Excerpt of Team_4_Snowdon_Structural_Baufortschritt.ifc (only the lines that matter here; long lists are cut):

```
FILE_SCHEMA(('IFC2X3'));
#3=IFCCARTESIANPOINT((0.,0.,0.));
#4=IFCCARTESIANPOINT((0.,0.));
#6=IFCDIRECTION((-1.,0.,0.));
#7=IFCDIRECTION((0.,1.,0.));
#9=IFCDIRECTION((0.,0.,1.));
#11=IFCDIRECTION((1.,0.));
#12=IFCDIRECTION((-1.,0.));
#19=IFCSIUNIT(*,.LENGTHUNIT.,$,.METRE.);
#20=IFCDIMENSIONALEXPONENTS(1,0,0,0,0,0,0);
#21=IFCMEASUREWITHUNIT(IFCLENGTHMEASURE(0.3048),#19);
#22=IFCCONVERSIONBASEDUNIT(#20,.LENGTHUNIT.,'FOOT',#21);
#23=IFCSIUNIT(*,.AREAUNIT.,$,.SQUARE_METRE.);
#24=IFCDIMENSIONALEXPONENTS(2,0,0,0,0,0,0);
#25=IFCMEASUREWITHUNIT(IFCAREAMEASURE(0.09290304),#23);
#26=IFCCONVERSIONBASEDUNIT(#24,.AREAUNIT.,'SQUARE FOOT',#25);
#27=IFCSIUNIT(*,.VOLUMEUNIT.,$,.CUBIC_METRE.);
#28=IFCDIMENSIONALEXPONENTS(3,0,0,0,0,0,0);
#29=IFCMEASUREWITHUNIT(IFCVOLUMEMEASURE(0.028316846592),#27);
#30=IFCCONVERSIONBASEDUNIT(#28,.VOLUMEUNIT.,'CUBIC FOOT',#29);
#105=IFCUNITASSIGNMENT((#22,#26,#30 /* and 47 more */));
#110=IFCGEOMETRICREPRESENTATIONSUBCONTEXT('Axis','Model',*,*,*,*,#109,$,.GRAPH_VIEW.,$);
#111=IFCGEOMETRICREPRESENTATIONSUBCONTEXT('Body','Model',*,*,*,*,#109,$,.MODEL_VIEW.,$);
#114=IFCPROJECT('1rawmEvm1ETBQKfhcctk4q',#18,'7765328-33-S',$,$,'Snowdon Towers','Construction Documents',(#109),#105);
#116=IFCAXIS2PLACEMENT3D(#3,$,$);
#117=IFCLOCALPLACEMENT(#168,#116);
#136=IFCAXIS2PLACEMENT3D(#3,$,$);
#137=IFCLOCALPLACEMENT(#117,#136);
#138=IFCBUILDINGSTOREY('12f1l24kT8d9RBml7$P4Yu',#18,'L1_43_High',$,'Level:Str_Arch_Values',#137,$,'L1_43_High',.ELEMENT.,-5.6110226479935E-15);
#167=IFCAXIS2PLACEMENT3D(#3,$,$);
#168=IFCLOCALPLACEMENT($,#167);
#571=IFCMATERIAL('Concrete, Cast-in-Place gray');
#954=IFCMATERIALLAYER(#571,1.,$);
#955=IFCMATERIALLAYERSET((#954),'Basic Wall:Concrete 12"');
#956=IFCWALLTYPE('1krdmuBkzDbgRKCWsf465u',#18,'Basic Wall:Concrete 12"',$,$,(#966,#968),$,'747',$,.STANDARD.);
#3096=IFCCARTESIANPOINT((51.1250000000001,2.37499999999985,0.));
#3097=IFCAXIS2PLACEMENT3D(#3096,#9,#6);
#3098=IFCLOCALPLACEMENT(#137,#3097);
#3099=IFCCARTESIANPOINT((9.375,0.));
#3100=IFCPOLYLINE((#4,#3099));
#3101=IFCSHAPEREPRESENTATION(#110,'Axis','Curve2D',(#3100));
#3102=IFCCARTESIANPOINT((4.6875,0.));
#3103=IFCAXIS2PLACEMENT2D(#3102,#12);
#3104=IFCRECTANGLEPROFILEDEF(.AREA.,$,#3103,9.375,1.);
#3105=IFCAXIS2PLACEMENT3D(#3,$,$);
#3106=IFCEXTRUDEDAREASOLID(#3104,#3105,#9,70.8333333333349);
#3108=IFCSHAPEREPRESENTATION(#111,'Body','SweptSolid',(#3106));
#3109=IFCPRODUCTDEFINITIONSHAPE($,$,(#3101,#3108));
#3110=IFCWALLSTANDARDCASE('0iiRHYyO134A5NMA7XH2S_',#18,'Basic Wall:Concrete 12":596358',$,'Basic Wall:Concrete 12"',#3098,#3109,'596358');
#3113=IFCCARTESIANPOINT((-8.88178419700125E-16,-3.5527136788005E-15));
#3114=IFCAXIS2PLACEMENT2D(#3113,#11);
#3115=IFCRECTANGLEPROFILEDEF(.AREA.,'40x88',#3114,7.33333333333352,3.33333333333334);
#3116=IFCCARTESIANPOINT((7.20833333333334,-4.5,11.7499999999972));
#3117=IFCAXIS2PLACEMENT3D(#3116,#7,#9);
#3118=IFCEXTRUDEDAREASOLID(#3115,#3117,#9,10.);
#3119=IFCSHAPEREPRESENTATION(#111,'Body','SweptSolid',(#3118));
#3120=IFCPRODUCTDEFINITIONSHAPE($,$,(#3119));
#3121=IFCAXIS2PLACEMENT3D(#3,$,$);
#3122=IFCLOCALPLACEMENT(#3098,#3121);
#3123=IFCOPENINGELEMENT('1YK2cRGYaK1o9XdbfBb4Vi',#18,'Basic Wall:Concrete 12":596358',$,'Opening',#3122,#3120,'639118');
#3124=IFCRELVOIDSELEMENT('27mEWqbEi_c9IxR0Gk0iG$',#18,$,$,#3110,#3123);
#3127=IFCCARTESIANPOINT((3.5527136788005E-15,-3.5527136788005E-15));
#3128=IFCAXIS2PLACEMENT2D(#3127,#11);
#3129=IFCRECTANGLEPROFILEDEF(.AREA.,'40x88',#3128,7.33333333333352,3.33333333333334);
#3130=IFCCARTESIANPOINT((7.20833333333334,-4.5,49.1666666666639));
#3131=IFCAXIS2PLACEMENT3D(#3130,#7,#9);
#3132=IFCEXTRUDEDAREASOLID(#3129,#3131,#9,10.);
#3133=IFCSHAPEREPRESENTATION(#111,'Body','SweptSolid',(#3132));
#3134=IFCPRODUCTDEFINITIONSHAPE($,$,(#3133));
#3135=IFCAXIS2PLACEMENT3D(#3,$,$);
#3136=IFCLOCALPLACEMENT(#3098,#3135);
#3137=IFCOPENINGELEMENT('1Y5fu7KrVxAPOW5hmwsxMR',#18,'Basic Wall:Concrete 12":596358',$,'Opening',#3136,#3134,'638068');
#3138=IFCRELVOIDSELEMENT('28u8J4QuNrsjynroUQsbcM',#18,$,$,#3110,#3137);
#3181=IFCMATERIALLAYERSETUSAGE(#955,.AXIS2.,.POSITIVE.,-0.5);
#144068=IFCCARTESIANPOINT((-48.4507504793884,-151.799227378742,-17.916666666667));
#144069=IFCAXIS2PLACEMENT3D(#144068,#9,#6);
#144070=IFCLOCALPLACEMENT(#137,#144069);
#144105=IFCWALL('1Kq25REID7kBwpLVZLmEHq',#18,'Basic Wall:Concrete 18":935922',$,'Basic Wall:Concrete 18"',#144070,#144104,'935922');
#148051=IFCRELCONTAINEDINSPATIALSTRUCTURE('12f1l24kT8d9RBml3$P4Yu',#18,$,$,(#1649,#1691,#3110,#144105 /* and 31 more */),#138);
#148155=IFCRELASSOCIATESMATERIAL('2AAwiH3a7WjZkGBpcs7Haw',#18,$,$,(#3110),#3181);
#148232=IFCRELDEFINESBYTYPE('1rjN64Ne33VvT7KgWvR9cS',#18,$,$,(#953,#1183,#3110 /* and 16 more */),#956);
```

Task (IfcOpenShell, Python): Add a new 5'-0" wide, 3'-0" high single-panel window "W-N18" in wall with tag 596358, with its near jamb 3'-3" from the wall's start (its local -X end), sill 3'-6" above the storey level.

```python
import numpy as np
import ifcopenshell
import ifcopenshell.api.feature
import ifcopenshell.api.geometry
import ifcopenshell.api.root
import ifcopenshell.api.spatial
import ifcopenshell.api.type
import ifcopenshell.geom
import ifcopenshell.util.element
import ifcopenshell.util.placement
import ifcopenshell.util.representation
import ifcopenshell.util.shape
import ifcopenshell.util.unit

model = ifcopenshell.open("Team_4_Snowdon_Structural_Baufortschritt.ifc")
unit_scale = ifcopenshell.util.unit.calculate_unit_scale(model)
settings = ifcopenshell.geom.settings()


def volume(element):
    """Net volume in cubic metres, openings subtracted."""
    shape = ifcopenshell.geom.create_shape(settings, element)
    return ifcopenshell.util.shape.get_volume(shape.geometry)


wall = model.by_guid("0iiRHYyO134A5NMA7XH2S_")
storey = ifcopenshell.util.element.get_container(wall, ifc_class="IfcBuildingStorey")
context = ifcopenshell.util.representation.get_context(model, "Model", "Body", "MODEL_VIEW")
before = volume(wall)

width, height, from_end, sill = 1.524, 0.9144, 0.9906, 1.0668  # metres

# The wall runs along its own X axis, and the end named is its -X end.
wall_shape = ifcopenshell.geom.create_shape(settings, wall)
x, y, z = ifcopenshell.util.shape.get_vertices(wall_shape.geometry).T
start = x.min() + from_end
face, thickness = float(y.min()), float(y.max() - y.min())
wall_matrix = ifcopenshell.util.placement.get_local_placement(wall.ObjectPlacement)
level = ifcopenshell.util.placement.get_local_placement(storey.ObjectPlacement)[2, 3]


def in_wall(x, y):
    """Placement at x, y metres in the wall's axes, at sill height."""
    matrix = wall_matrix.copy()
    matrix[:, 3] = wall_matrix @ np.array([x / unit_scale, y / unit_scale, 0.0, 1.0])
    matrix[2, 3] = level + sill / unit_scale
    return matrix


# Opening: a box that overshoots both wall faces by 50 mm.
opening = ifcopenshell.api.root.create_entity(model, ifc_class="IfcOpeningElement")
box = ifcopenshell.api.geometry.add_wall_representation(
    model, context=context, length=width, height=height, thickness=thickness + 0.1
)
ifcopenshell.api.geometry.assign_representation(model, product=opening, representation=box)
ifcopenshell.api.geometry.edit_object_placement(model, product=opening, matrix=in_wall(start, face - 0.05), is_si=False)
ifcopenshell.api.feature.add_feature(model, feature=opening, element=wall)

window = ifcopenshell.api.root.create_entity(model, ifc_class="IfcWindow", name="W-N18")
window.OverallWidth, window.OverallHeight = width / unit_scale, height / unit_scale
body = ifcopenshell.api.geometry.add_window_representation(
    model,
    context=context,
    overall_width=window.OverallWidth,
    overall_height=window.OverallHeight,
    partition_type="SINGLE_PANEL",
)
ifcopenshell.api.geometry.assign_representation(model, product=window, representation=body)
ifcopenshell.api.spatial.assign_container(model, products=[window], relating_structure=storey)
fills = ifcopenshell.api.feature.add_filling(model, opening=opening, element=window)
fills.OwnerHistory = window.OwnerHistory  # required in IFC2X3

# IFC2X3 keeps the operation on the window style.
style = ifcopenshell.api.root.create_entity(model, ifc_class="IfcWindowStyle", name="W-N18")
style.OperationType, style.ConstructionType = "SINGLE_PANEL", "NOTDEFINED"
style.ParameterTakesPrecedence = style.Sizeable = False
ifcopenshell.api.type.assign_type(model, related_objects=[window], relating_type=style)

# Centre the window in the wall's thickness.
ifcopenshell.api.geometry.edit_object_placement(model, product=window, matrix=in_wall(start, face), is_si=False)
window_shape = ifcopenshell.geom.create_shape(settings, window)
depth = ifcopenshell.util.shape.get_vertices(window_shape.geometry)[:, 1]
offset = face + thickness / 2 - (depth.min() + depth.max()) / 2
ifcopenshell.api.geometry.edit_object_placement(model, product=window, matrix=in_wall(start, offset), is_si=False)

after = volume(wall)

print(f"wall volume {before:.3f} -> {after:.3f} m3")

model.write("Team_4_Snowdon_Structural_Baufortschritt_updated.ifc")
```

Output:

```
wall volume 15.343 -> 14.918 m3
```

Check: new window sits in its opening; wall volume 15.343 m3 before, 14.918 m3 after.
